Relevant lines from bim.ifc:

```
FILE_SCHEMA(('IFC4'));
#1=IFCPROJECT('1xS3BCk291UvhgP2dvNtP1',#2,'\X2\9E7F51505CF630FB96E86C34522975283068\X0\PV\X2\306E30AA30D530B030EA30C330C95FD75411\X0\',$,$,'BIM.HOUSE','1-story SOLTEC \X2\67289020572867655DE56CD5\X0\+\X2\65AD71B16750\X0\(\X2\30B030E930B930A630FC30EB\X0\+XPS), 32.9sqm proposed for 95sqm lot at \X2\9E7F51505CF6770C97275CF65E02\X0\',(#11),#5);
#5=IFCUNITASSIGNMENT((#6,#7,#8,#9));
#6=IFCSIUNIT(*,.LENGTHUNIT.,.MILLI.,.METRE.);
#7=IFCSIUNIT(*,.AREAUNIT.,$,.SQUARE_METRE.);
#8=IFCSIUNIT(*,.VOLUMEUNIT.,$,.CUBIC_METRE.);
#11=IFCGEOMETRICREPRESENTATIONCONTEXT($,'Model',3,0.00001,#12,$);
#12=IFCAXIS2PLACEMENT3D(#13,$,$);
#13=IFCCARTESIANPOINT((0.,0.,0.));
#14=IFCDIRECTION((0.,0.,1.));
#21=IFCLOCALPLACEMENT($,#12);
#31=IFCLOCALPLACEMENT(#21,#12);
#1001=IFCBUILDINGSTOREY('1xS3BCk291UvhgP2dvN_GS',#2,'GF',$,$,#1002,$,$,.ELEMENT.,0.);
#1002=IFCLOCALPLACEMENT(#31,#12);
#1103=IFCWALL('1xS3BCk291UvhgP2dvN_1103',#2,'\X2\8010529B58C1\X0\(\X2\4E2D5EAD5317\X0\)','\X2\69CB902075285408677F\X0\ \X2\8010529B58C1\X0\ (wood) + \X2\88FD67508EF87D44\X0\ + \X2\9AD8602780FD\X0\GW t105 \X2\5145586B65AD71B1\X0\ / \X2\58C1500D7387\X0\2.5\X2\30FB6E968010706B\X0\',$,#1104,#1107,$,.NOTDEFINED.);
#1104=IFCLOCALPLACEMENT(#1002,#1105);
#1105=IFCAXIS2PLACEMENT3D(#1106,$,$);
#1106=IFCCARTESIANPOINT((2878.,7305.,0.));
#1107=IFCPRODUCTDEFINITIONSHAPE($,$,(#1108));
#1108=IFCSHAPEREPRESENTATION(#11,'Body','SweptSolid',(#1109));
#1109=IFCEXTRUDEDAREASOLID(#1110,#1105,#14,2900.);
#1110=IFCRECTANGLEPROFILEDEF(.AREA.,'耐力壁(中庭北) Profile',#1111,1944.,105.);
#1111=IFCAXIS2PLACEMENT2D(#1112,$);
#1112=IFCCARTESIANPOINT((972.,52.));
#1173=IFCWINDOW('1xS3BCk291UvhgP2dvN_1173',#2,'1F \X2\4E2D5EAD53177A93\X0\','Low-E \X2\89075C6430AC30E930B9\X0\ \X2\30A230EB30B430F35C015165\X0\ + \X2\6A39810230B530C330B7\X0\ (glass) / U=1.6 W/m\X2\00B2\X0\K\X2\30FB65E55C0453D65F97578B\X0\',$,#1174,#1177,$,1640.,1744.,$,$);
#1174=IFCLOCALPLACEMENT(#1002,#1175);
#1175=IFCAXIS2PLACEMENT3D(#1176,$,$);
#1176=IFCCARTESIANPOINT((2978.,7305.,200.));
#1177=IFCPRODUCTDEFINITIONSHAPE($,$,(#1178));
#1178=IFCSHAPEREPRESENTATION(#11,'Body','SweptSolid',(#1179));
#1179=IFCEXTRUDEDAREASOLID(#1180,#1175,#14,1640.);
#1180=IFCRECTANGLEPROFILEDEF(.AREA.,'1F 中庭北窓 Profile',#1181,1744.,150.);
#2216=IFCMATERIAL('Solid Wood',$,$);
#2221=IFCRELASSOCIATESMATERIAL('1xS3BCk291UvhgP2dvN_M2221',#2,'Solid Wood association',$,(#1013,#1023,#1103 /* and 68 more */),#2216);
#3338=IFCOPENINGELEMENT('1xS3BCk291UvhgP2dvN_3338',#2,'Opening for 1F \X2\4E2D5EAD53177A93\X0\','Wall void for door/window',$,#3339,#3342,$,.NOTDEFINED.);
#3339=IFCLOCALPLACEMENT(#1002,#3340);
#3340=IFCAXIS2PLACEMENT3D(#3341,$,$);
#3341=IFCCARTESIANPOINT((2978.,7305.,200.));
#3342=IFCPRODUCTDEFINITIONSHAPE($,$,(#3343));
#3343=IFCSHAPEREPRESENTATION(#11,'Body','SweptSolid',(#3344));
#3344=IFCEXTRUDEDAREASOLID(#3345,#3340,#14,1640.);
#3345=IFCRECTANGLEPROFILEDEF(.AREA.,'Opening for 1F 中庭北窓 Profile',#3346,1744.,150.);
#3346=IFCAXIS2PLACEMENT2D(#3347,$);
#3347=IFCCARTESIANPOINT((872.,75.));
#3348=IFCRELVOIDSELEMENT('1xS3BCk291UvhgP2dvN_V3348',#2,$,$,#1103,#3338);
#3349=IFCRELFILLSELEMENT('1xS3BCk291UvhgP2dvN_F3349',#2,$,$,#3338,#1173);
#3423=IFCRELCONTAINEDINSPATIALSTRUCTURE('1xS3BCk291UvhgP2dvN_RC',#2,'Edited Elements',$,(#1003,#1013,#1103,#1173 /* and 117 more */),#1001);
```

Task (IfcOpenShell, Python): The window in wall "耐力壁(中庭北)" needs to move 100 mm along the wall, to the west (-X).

```python
import ifcopenshell
import ifcopenshell.api.geometry
import ifcopenshell.util.placement

model = ifcopenshell.open("bim.ifc")

window = model.by_guid("1xS3BCk291UvhgP2dvN_1173")
opening = window.FillsVoids[0].RelatingOpeningElement
wall = opening.VoidsElements[0].RelatingBuildingElement

wall_matrix = ifcopenshell.util.placement.get_local_placement(wall.ObjectPlacement)
shift = wall_matrix[:3, 0] * -100.0
before = ifcopenshell.util.placement.get_local_placement(window.ObjectPlacement)[:3, 3].copy()

# The window is not placed relative to its opening, so move both.
for product in (opening, window):
    matrix = ifcopenshell.util.placement.get_local_placement(product.ObjectPlacement)
    matrix[:3, 3] += shift
    ifcopenshell.api.geometry.edit_object_placement(model, product=product, matrix=matrix, is_si=False)

after = ifcopenshell.util.placement.get_local_placement(window.ObjectPlacement)[:3, 3]
print("window moved by", (after - before).round(3) + 0.0)

model.write("bim_v2.ifc")
```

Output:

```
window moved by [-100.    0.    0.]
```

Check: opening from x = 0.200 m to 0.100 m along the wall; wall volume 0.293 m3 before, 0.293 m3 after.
